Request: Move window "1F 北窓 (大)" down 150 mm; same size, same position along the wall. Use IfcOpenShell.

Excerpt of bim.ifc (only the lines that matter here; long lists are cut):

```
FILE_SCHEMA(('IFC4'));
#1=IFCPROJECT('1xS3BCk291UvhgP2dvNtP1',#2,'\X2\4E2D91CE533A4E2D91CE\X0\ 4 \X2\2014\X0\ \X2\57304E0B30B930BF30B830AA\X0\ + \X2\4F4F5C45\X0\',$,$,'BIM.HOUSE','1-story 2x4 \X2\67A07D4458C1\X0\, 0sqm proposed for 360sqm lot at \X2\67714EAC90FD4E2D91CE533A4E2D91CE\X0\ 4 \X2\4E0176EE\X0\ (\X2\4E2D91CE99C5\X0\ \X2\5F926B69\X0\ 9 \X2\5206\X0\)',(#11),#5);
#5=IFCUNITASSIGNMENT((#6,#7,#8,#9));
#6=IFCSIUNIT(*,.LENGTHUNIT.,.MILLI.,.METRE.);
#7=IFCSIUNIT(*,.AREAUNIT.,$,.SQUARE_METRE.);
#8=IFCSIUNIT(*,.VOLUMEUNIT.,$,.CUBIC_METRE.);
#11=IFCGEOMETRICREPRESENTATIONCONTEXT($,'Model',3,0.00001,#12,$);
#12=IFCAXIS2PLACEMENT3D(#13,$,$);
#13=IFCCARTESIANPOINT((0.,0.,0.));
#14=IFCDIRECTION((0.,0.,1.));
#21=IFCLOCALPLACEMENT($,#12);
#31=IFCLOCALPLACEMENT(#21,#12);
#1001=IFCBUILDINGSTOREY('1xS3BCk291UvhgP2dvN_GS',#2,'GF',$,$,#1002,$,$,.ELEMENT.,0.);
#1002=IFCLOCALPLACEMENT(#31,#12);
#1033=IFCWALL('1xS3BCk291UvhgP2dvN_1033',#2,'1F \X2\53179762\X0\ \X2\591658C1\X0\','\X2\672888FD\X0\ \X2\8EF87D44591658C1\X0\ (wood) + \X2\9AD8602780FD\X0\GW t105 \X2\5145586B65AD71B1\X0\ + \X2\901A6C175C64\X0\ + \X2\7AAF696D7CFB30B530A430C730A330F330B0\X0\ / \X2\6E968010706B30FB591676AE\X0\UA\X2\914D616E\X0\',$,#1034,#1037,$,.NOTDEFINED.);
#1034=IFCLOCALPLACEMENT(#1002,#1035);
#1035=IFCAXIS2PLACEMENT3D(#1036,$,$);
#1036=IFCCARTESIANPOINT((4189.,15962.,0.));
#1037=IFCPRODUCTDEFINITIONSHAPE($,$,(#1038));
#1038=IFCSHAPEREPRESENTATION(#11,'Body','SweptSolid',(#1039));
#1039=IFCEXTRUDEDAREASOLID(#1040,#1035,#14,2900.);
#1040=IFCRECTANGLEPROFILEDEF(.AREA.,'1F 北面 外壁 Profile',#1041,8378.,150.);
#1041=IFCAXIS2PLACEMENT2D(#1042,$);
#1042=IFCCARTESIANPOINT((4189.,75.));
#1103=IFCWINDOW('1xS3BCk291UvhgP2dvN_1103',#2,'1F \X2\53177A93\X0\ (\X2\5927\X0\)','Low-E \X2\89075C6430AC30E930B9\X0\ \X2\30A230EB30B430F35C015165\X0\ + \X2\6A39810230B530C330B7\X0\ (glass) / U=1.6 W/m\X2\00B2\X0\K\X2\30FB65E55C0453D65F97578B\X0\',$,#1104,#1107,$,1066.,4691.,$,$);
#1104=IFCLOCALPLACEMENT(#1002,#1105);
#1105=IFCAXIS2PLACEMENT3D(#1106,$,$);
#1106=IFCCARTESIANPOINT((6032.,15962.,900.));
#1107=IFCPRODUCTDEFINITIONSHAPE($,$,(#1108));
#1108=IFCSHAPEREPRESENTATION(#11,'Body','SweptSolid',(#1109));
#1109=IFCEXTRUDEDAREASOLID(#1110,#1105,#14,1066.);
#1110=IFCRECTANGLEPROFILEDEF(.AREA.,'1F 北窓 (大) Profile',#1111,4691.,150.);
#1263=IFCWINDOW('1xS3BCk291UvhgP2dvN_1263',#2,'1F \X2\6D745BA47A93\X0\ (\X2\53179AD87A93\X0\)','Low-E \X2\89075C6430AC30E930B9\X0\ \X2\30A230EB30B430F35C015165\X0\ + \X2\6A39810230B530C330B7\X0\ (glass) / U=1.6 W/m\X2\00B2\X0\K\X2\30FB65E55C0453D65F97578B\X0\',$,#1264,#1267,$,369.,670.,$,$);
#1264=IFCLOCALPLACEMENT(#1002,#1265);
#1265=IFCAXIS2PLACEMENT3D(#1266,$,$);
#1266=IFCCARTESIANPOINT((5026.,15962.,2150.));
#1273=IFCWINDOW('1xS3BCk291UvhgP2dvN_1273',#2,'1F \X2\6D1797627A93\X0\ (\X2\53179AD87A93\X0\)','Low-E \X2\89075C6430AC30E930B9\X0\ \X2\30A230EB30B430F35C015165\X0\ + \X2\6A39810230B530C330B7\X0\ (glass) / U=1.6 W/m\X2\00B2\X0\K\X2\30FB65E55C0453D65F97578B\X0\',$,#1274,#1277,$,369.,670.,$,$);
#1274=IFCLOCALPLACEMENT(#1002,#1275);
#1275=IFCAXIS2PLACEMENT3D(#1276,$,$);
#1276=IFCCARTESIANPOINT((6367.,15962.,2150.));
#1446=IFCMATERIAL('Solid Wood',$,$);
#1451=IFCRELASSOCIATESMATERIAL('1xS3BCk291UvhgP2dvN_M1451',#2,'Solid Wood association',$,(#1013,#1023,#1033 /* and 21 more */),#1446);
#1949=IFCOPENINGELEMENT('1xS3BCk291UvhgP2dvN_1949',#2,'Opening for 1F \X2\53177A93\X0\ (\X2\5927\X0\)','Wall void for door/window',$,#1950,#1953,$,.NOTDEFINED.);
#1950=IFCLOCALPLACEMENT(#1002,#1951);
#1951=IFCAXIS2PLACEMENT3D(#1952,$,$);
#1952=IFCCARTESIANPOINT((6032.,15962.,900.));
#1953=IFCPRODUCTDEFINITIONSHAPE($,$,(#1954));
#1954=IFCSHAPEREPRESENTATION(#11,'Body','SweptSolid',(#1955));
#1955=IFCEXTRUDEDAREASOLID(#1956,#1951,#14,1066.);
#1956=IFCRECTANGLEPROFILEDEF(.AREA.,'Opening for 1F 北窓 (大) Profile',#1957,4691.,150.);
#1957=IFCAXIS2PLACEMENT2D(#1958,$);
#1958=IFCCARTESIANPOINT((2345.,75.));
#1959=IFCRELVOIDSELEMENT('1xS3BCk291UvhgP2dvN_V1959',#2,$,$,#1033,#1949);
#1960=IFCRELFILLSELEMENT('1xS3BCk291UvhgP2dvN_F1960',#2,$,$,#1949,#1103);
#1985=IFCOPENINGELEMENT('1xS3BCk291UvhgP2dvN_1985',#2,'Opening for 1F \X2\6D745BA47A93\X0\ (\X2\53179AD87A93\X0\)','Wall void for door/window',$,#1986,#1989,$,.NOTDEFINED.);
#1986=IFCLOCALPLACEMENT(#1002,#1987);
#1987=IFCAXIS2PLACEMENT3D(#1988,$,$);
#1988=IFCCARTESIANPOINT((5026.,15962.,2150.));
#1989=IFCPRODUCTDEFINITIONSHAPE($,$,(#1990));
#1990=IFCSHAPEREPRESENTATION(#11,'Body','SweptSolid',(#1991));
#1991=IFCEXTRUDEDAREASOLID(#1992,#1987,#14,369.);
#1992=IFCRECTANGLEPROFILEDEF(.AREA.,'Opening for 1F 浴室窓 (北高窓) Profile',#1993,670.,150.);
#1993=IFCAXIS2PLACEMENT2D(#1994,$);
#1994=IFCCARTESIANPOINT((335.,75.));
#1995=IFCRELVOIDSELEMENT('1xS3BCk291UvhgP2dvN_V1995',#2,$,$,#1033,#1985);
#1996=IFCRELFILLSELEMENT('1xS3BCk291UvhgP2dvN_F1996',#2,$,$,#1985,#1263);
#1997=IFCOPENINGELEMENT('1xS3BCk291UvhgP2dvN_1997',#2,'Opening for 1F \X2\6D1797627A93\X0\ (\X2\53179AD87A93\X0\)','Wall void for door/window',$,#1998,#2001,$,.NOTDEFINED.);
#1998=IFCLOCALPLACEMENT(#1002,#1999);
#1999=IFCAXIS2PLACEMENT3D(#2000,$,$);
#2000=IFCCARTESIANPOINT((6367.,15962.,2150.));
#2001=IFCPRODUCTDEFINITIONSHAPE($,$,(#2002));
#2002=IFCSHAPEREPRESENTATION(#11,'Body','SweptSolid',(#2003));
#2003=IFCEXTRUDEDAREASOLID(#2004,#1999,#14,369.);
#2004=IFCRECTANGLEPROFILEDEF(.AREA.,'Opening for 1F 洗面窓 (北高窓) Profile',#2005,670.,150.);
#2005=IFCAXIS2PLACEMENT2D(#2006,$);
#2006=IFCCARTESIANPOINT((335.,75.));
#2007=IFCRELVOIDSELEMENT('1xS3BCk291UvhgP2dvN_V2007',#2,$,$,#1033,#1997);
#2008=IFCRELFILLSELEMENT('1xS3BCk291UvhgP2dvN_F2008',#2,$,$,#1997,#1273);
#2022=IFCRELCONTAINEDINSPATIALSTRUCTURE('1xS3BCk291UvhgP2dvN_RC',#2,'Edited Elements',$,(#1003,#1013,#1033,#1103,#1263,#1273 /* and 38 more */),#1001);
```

```python
import numpy as np
import ifcopenshell
import ifcopenshell.api.geometry
import ifcopenshell.util.placement
import ifcopenshell.util.unit

model = ifcopenshell.open("bim.ifc")
unit_scale = ifcopenshell.util.unit.calculate_unit_scale(model)

window = model.by_id(1103)
opening = window.FillsVoids[0].RelatingOpeningElement
dz = -150.0

shift = np.array([0.0, 0.0, dz])
# The window is not placed relative to its opening, so move both.
for product in (opening, window):
    matrix = ifcopenshell.util.placement.get_local_placement(product.ObjectPlacement)
    matrix[:3, 3] += shift
    ifcopenshell.api.geometry.edit_object_placement(model, product=product, matrix=matrix, is_si=False)

print(f"moved by {dz * unit_scale:+.3f} m")

model.write("bim_rev.ifc")
```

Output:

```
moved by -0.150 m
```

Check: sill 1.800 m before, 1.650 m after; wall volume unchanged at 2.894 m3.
